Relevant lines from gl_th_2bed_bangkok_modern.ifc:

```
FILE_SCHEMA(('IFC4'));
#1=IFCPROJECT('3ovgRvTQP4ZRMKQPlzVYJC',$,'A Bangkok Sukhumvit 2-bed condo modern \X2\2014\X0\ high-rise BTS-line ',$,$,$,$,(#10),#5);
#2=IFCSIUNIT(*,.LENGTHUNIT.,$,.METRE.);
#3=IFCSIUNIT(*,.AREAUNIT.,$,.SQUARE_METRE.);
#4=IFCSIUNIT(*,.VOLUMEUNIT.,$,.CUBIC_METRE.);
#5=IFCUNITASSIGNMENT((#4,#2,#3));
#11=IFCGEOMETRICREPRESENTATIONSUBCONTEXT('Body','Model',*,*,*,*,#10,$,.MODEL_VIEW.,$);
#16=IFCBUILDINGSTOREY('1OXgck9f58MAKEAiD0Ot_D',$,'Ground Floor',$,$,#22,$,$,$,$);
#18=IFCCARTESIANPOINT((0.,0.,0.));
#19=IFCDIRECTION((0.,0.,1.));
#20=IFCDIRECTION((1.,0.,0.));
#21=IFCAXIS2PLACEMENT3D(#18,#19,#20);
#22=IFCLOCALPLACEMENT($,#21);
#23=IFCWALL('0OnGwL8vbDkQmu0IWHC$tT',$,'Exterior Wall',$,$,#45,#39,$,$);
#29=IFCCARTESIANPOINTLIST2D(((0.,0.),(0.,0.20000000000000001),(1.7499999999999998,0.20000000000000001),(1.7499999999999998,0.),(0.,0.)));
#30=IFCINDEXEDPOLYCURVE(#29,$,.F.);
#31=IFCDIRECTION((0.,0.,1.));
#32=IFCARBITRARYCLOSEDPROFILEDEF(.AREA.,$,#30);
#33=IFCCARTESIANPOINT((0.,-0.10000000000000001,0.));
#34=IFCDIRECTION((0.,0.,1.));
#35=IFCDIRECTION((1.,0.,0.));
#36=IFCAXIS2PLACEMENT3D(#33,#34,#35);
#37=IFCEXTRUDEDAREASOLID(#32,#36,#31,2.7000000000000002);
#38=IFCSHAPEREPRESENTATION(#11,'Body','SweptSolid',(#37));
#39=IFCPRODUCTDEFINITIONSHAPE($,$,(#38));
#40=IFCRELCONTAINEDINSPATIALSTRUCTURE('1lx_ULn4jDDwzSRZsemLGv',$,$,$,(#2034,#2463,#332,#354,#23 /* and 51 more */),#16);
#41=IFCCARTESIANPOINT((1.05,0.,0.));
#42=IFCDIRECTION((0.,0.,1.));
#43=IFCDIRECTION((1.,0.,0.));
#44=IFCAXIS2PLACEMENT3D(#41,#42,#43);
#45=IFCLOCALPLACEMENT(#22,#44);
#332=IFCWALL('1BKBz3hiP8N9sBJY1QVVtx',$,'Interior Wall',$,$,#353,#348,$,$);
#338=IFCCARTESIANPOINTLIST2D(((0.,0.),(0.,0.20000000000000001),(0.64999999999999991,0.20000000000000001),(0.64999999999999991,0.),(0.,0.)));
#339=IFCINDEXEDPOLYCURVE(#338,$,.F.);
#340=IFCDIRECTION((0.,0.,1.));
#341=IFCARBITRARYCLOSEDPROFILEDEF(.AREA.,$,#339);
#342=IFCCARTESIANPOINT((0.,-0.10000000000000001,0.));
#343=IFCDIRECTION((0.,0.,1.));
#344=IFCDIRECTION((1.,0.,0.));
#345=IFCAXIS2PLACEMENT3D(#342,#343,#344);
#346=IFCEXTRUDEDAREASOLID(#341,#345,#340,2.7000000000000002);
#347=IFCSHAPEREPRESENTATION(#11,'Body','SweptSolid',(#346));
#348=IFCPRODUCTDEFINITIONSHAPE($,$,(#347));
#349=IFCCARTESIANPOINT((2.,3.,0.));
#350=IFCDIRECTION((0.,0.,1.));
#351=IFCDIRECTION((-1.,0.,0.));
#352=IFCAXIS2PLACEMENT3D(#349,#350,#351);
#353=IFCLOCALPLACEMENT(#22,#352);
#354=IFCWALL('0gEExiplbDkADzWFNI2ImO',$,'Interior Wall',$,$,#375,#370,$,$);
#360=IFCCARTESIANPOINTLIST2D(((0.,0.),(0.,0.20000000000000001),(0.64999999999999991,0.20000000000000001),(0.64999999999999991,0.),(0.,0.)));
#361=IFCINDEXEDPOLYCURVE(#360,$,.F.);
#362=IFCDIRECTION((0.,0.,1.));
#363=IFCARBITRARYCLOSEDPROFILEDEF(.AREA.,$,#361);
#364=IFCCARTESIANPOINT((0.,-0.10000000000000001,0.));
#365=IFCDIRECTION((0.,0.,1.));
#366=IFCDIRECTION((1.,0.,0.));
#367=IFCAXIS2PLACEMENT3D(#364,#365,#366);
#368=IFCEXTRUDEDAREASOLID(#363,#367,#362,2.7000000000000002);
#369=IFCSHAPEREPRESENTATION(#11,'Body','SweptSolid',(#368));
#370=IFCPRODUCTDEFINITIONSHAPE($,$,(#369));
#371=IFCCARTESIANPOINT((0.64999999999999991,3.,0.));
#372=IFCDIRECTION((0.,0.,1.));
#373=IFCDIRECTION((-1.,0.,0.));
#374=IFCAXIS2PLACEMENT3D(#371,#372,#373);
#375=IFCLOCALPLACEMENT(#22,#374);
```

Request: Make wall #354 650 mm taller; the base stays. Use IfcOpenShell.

```python
import ifcopenshell
import ifcopenshell.geom
import ifcopenshell.util.representation
import ifcopenshell.util.shape

model = ifcopenshell.open("gl_th_2bed_bangkok_modern.ifc")
settings = ifcopenshell.geom.settings()


def volume(element):
    """Net volume in cubic metres, openings subtracted."""
    shape = ifcopenshell.geom.create_shape(settings, element)
    return ifcopenshell.util.shape.get_volume(shape.geometry)


wall = model.by_guid("0gEExiplbDkADzWFNI2ImO")
before = volume(wall)

body = ifcopenshell.util.representation.get_representation(wall, "Model", "Body")
solid = body.Items[0]
old_height = solid.Depth
solid.Depth += 0.65
after = volume(wall)

print(f"height {old_height:g} -> {solid.Depth:g}, volume {before:.3f} -> {after:.3f} m3")

model.write("gl_th_2bed_bangkok_modern_updated.ifc")
```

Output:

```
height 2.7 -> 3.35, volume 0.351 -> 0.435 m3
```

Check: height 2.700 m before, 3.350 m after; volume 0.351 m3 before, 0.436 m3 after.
